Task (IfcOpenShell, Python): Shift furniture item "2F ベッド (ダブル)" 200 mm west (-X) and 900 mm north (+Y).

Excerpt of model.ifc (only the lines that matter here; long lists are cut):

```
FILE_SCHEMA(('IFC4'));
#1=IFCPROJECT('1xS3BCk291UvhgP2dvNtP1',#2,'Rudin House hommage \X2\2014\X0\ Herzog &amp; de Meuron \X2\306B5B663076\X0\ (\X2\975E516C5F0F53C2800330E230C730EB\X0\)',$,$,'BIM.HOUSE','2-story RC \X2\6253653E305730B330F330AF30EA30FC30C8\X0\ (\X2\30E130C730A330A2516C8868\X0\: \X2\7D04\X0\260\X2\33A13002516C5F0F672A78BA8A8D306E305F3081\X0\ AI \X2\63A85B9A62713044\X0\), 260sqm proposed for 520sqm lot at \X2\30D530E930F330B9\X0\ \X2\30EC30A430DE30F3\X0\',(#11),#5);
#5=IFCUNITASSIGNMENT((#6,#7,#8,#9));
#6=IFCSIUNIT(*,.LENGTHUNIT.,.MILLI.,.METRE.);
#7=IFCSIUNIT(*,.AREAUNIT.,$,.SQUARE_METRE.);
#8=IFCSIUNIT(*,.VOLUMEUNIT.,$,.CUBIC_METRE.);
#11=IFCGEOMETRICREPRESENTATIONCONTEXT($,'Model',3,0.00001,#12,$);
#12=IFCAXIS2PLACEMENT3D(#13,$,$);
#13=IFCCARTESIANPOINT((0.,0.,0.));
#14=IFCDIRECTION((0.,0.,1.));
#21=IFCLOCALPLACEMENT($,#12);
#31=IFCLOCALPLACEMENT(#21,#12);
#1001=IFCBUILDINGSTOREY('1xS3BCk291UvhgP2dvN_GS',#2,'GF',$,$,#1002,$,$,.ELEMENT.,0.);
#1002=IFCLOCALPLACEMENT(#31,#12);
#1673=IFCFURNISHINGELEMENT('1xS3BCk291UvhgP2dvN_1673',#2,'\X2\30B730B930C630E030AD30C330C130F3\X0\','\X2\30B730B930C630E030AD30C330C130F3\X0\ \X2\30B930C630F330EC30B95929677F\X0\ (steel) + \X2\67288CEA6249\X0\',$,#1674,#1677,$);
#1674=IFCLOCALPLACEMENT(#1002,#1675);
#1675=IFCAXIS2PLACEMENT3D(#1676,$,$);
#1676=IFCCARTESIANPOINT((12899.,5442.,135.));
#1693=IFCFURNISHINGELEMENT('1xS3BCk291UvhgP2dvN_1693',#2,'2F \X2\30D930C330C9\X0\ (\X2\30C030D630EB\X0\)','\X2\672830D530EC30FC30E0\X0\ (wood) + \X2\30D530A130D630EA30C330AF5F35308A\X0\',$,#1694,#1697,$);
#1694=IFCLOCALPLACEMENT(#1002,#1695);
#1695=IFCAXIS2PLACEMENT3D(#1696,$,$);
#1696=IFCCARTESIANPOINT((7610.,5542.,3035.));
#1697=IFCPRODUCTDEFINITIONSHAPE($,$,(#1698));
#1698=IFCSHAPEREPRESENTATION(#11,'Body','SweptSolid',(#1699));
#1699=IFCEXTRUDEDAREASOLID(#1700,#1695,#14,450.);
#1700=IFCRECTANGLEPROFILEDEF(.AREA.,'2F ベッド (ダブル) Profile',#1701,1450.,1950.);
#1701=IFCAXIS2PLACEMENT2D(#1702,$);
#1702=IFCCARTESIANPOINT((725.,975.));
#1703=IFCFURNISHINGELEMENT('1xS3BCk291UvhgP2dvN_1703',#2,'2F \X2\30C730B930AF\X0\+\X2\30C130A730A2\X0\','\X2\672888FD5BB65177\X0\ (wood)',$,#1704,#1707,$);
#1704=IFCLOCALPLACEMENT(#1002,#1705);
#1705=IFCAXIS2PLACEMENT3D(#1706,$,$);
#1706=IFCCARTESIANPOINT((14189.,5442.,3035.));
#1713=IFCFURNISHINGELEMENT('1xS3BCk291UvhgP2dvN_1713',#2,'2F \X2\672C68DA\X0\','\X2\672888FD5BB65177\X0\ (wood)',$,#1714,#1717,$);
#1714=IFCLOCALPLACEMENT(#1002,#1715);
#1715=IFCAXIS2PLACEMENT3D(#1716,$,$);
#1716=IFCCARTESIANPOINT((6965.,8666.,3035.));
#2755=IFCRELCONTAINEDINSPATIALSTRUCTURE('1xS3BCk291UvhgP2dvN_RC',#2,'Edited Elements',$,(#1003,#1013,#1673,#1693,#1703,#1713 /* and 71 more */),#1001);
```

```python
import ifcopenshell
import ifcopenshell.api.geometry
import ifcopenshell.util.placement
import ifcopenshell.util.unit

model = ifcopenshell.open("model.ifc")
unit_scale = ifcopenshell.util.unit.calculate_unit_scale(model)

item = model.by_id(1693)
matrix = ifcopenshell.util.placement.get_local_placement(item.ObjectPlacement)
matrix[0, 3] -= 0.2 / unit_scale
matrix[1, 3] += 0.9 / unit_scale
ifcopenshell.api.geometry.edit_object_placement(model, product=item, matrix=matrix, is_si=False)

print(ifcopenshell.util.placement.get_local_placement(item.ObjectPlacement).round(3) + 0.0)

model.write("model_edited.ifc")
```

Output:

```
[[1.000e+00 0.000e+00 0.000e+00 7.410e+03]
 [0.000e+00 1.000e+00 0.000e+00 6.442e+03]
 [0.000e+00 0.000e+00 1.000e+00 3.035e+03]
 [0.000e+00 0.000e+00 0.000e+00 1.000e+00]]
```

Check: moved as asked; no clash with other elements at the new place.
